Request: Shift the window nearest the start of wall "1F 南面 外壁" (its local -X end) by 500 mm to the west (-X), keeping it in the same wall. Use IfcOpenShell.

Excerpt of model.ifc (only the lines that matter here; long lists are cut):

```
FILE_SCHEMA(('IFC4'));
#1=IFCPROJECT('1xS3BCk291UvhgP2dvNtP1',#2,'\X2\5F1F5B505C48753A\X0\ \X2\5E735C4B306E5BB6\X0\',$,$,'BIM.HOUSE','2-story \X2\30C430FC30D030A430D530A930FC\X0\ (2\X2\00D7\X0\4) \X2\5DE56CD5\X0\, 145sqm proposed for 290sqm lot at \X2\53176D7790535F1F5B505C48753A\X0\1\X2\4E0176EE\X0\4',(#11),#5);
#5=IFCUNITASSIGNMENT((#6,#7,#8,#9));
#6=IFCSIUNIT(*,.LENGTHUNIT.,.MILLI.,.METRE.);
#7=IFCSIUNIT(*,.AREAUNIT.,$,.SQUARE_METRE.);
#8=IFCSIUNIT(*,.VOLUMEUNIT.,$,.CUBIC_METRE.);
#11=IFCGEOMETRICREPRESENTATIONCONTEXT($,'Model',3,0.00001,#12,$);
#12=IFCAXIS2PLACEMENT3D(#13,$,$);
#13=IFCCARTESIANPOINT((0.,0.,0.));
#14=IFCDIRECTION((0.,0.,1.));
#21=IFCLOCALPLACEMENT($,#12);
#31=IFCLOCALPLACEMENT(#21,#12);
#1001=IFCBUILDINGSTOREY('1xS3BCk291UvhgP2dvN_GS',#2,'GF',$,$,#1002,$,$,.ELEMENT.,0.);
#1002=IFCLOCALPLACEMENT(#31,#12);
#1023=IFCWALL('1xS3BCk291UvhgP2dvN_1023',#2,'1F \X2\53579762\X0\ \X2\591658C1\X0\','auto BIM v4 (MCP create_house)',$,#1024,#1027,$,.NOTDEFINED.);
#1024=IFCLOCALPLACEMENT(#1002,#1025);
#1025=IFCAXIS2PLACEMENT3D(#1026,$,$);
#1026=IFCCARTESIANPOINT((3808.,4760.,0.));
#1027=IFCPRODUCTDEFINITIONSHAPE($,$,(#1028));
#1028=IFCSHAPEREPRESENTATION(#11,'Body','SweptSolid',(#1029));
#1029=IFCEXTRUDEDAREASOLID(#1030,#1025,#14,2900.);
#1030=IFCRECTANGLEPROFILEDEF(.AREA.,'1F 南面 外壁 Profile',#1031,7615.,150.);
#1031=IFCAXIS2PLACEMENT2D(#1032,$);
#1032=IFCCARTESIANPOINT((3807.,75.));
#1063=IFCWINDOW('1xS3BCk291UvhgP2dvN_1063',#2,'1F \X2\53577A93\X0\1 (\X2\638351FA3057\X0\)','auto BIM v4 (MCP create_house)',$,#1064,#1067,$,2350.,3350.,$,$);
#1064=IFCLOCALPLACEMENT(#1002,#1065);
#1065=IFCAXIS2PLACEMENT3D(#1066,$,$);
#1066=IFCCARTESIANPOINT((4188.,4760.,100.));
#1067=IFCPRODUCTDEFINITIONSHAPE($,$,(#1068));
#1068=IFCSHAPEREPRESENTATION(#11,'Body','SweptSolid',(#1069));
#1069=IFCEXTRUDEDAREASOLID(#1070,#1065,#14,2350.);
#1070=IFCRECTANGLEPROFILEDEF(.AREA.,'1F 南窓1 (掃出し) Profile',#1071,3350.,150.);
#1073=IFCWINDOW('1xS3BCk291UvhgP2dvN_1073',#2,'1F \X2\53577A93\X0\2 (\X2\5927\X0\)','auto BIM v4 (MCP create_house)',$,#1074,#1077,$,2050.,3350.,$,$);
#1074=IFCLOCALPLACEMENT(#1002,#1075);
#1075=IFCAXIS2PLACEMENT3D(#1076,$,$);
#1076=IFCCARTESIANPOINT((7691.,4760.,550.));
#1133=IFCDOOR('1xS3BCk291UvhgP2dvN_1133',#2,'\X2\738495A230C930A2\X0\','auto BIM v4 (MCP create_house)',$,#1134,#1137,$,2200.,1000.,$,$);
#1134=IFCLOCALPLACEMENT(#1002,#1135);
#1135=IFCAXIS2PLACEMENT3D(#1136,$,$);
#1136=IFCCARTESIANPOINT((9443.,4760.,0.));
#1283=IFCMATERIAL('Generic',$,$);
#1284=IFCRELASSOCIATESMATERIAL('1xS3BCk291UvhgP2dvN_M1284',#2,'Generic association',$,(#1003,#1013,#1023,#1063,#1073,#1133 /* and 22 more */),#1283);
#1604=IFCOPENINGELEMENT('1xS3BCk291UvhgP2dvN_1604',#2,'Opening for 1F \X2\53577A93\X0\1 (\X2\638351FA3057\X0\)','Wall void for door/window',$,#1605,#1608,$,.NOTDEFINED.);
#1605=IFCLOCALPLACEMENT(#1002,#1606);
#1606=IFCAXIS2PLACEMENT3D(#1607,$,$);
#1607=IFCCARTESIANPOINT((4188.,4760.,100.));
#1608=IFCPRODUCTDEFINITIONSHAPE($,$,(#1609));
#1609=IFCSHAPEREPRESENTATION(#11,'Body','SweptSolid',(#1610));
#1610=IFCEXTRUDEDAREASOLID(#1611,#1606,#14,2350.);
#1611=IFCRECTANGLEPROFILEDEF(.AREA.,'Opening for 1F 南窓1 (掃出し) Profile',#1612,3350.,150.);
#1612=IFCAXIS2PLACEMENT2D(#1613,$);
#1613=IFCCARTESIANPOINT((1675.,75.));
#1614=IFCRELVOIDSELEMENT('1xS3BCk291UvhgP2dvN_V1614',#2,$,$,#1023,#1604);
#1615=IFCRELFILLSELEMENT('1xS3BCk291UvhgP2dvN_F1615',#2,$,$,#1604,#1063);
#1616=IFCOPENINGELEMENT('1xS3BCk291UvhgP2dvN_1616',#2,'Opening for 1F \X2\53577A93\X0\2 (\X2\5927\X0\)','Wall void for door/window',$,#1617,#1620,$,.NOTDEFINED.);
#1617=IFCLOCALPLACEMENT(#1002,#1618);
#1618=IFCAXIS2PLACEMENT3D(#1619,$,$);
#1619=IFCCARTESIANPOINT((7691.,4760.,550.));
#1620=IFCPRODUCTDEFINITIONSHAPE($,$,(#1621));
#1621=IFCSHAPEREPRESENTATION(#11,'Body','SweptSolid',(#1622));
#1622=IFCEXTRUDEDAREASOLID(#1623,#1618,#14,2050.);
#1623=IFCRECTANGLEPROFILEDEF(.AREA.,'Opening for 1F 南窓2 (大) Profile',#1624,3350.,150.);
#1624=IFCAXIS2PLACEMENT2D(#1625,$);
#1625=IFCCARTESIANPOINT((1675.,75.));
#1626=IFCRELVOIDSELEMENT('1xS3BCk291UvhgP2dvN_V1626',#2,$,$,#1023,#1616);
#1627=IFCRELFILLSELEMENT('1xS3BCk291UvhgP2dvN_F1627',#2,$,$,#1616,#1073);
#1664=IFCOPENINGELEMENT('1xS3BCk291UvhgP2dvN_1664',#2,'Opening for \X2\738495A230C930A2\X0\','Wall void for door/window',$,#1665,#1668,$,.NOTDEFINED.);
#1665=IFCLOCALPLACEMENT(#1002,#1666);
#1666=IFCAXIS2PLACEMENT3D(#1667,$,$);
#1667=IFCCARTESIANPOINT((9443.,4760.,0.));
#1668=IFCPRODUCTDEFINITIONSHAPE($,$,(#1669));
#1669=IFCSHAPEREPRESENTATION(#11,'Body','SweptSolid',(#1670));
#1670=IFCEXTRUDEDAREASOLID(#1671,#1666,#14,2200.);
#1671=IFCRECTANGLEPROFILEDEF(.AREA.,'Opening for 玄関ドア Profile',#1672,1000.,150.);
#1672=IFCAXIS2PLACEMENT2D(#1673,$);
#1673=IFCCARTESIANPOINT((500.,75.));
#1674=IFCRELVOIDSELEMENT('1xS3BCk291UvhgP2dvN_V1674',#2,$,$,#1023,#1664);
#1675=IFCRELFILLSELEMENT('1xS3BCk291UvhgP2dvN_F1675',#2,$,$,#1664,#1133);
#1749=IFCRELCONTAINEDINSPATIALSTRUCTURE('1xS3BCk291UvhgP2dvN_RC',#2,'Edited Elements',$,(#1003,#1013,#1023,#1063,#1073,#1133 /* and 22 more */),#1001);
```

```python
import ifcopenshell
import ifcopenshell.api.geometry
import ifcopenshell.util.placement
import ifcopenshell.util.unit

model = ifcopenshell.open("model.ifc")
unit_scale = ifcopenshell.util.unit.calculate_unit_scale(model)

window = model.by_guid("1xS3BCk291UvhgP2dvN_1063")
opening = window.FillsVoids[0].RelatingOpeningElement
wall = opening.VoidsElements[0].RelatingBuildingElement

wall_matrix = ifcopenshell.util.placement.get_local_placement(wall.ObjectPlacement)
shift = wall_matrix[:3, 0] * -0.5 / unit_scale
before = ifcopenshell.util.placement.get_local_placement(window.ObjectPlacement)[:3, 3].copy()

# The window is not placed relative to its opening, so move both.
for product in (opening, window):
    matrix = ifcopenshell.util.placement.get_local_placement(product.ObjectPlacement)
    matrix[:3, 3] += shift
    ifcopenshell.api.geometry.edit_object_placement(model, product=product, matrix=matrix, is_si=False)

after = ifcopenshell.util.placement.get_local_placement(window.ObjectPlacement)[:3, 3]
print("window moved by", (after - before).round(3) + 0.0)

model.write("model-out.ifc")
```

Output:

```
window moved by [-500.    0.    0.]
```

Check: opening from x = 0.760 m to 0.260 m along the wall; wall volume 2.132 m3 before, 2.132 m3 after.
